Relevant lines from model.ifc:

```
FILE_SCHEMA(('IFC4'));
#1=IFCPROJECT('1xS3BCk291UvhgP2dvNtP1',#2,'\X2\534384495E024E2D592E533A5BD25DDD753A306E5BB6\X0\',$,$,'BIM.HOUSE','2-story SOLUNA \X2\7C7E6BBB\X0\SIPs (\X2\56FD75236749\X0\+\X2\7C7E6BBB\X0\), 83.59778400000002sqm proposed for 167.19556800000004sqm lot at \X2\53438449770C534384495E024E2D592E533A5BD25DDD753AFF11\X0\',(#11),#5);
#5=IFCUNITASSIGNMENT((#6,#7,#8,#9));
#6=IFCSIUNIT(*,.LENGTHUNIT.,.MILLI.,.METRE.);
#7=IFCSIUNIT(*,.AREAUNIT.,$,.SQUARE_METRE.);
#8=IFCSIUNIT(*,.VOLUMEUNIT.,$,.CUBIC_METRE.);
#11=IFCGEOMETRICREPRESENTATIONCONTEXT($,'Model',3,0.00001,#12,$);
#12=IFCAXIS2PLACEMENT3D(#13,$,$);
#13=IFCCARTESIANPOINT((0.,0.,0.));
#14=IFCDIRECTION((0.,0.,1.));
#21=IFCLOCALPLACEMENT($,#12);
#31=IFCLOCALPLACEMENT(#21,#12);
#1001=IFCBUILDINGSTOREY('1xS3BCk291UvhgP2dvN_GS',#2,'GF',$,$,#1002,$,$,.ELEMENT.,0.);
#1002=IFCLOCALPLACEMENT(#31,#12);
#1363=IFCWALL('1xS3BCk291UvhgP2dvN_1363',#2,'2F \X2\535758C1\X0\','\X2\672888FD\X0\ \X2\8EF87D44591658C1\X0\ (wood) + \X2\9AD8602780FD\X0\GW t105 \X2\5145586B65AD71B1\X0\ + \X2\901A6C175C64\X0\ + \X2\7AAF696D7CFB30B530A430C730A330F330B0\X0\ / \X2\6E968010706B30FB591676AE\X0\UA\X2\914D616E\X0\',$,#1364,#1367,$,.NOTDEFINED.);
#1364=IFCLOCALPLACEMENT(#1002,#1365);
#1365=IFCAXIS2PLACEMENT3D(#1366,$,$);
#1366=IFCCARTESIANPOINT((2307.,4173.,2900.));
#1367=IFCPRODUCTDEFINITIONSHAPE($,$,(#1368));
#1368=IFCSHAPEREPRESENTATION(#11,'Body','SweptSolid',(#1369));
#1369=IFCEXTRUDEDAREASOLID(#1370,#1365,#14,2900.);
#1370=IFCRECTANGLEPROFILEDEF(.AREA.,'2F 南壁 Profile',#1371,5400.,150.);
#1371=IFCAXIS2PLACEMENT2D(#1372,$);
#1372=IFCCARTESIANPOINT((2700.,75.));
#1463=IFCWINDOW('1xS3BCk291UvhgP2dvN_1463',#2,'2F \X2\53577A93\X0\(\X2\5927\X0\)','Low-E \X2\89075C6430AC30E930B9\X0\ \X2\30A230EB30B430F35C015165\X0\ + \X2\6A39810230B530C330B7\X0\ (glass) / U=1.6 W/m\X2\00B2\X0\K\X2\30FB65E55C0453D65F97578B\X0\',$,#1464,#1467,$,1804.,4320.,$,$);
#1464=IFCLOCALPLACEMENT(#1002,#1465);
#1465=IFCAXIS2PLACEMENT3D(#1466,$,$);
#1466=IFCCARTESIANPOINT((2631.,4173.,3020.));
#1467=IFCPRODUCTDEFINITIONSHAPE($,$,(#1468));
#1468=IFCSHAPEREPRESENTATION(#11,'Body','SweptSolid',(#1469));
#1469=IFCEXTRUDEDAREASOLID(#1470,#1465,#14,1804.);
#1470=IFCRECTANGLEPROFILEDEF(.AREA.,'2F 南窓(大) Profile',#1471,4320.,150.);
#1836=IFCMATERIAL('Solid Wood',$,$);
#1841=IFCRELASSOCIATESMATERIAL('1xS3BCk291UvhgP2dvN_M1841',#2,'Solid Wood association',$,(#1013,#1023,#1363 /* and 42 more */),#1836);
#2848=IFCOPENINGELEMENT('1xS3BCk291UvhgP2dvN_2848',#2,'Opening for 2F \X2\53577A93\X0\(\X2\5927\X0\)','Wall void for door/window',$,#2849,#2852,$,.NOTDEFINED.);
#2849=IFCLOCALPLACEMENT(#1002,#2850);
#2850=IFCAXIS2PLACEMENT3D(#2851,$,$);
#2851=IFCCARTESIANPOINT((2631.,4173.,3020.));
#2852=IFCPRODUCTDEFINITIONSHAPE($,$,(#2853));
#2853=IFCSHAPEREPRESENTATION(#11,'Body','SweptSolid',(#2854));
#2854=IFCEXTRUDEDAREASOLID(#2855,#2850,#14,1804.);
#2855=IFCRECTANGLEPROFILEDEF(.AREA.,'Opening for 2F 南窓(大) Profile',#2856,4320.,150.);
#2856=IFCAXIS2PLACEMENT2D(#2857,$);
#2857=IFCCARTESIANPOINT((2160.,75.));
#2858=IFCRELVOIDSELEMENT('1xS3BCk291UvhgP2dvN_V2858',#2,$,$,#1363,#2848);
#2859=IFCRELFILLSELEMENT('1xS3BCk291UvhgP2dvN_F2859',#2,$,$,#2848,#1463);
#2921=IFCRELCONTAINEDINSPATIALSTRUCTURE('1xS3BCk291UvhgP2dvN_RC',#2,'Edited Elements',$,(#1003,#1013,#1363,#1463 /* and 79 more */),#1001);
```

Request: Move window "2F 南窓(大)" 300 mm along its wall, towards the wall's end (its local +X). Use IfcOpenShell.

```python
import ifcopenshell
import ifcopenshell.api.geometry
import ifcopenshell.util.placement
import ifcopenshell.util.unit

model = ifcopenshell.open("model.ifc")
unit_scale = ifcopenshell.util.unit.calculate_unit_scale(model)

window = model.by_id(1463)
opening = window.FillsVoids[0].RelatingOpeningElement
wall = opening.VoidsElements[0].RelatingBuildingElement

wall_matrix = ifcopenshell.util.placement.get_local_placement(wall.ObjectPlacement)
shift = wall_matrix[:3, 0] * 0.3 / unit_scale
before = ifcopenshell.util.placement.get_local_placement(window.ObjectPlacement)[:3, 3].copy()

# The window is not placed relative to its opening, so move both.
for product in (opening, window):
    matrix = ifcopenshell.util.placement.get_local_placement(product.ObjectPlacement)
    matrix[:3, 3] += shift
    ifcopenshell.api.geometry.edit_object_placement(model, product=product, matrix=matrix, is_si=False)

after = ifcopenshell.util.placement.get_local_placement(window.ObjectPlacement)[:3, 3]
print("window moved by", (after - before).round(3) + 0.0)

model.write("model_rev.ifc")
```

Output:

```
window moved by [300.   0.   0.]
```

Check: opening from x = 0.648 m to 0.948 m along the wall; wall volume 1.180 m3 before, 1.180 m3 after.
